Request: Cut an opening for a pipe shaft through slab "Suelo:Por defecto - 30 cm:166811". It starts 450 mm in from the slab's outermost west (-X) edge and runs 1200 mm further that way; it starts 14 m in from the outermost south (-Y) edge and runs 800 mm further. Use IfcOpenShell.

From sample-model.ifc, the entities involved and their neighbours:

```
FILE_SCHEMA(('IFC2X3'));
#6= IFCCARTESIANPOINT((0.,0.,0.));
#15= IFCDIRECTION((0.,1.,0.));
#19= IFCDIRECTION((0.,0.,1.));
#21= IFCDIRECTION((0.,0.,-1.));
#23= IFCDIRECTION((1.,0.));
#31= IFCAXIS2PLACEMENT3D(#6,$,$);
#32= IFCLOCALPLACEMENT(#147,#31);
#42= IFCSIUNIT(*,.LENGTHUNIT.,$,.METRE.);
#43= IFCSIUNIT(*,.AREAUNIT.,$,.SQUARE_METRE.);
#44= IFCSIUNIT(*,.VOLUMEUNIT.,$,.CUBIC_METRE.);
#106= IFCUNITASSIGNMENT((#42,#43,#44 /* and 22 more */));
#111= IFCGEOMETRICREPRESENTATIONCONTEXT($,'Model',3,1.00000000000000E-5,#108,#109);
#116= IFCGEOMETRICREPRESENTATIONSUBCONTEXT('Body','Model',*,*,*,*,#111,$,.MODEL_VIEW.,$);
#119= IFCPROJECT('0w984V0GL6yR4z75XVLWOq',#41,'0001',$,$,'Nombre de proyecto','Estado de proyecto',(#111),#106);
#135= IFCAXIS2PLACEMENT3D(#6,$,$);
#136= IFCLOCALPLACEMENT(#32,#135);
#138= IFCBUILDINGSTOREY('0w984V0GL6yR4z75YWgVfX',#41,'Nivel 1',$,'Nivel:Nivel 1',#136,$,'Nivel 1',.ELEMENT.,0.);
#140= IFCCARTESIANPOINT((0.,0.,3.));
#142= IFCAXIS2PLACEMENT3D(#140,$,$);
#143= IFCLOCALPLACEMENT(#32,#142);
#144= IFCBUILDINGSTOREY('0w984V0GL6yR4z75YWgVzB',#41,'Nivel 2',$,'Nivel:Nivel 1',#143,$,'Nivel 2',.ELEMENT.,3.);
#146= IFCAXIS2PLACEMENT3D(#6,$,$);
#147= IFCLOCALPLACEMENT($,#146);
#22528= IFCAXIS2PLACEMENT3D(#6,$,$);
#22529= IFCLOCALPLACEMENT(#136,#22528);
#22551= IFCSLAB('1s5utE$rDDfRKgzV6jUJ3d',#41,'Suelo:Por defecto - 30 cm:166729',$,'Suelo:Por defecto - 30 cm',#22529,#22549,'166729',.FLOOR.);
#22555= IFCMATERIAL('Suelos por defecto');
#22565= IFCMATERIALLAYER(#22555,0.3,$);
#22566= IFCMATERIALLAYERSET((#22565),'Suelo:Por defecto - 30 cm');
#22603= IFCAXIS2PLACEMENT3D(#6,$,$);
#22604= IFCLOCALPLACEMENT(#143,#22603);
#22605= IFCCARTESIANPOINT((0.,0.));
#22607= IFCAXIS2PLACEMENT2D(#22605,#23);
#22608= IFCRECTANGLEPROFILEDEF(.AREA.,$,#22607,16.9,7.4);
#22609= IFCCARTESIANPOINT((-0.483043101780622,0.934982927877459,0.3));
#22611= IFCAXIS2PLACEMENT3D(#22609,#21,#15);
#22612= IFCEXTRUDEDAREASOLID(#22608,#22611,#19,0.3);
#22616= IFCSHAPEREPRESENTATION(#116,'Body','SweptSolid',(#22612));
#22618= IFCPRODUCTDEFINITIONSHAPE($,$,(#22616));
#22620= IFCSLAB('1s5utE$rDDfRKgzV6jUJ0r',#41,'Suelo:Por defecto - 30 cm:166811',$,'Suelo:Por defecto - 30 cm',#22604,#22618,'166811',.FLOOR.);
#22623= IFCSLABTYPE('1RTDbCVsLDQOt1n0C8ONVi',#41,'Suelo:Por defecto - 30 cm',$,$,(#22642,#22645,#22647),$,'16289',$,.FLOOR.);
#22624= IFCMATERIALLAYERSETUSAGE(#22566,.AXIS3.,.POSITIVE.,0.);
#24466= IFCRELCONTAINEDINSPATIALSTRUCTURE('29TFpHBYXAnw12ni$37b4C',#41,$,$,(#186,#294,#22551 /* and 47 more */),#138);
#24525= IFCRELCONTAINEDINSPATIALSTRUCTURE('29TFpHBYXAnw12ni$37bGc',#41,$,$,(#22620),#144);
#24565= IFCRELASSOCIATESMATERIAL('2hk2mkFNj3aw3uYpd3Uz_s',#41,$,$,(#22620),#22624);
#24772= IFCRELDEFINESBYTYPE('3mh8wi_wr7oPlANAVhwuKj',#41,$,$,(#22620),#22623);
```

```python
import numpy as np
import ifcopenshell
import ifcopenshell.api.feature
import ifcopenshell.api.geometry
import ifcopenshell.api.root
import ifcopenshell.geom
import ifcopenshell.util.placement
import ifcopenshell.util.representation
import ifcopenshell.util.shape
import ifcopenshell.util.unit

model = ifcopenshell.open("sample-model.ifc")
unit_scale = ifcopenshell.util.unit.calculate_unit_scale(model)
settings = ifcopenshell.geom.settings()


def volume(element):
    """Net volume in cubic metres, openings subtracted."""
    shape = ifcopenshell.geom.create_shape(settings, element)
    return ifcopenshell.util.shape.get_volume(shape.geometry)


slab = model.by_id(22620)
before = volume(slab)

# Extent in the slab's own axes, in metres. The edges named are its -X and -Y sides.
slab_shape = ifcopenshell.geom.create_shape(settings, slab)
vertices = ifcopenshell.util.shape.get_vertices(slab_shape.geometry)
x_min, y_min, bottom = vertices.min(axis=0)
top = vertices[:, 2].max()

opening = ifcopenshell.api.root.create_entity(model, ifc_class="IfcOpeningElement", name="Pipe shaft opening")
context = ifcopenshell.util.representation.get_context(model, "Model", "Body", "MODEL_VIEW")
width, depth = 1.2, 0.8
outline = [(0.0, 0.0), (width, 0.0), (width, depth), (0.0, depth), (0.0, 0.0)]
# Overshoot both faces by 50 mm so the cut is clean.
shape = ifcopenshell.api.geometry.add_slab_representation(
    model, context=context, depth=top - bottom + 0.1, polyline=outline
)
ifcopenshell.api.geometry.assign_representation(model, product=opening, representation=shape)

matrix = ifcopenshell.util.placement.get_local_placement(slab.ObjectPlacement)
matrix[:, 3] = matrix @ np.append(np.array([x_min + 0.45, y_min + 14, bottom - 0.05]) / unit_scale, 1.0)
ifcopenshell.api.geometry.edit_object_placement(model, product=opening, matrix=matrix, is_si=False)
ifcopenshell.api.feature.add_feature(model, feature=opening, element=slab)

after = volume(slab)

print(f"slab volume {before:.3f} -> {after:.3f} m3")

model.write("sample-model_v2.ifc")
```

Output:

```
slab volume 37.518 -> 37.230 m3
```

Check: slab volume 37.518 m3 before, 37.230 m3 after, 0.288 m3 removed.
